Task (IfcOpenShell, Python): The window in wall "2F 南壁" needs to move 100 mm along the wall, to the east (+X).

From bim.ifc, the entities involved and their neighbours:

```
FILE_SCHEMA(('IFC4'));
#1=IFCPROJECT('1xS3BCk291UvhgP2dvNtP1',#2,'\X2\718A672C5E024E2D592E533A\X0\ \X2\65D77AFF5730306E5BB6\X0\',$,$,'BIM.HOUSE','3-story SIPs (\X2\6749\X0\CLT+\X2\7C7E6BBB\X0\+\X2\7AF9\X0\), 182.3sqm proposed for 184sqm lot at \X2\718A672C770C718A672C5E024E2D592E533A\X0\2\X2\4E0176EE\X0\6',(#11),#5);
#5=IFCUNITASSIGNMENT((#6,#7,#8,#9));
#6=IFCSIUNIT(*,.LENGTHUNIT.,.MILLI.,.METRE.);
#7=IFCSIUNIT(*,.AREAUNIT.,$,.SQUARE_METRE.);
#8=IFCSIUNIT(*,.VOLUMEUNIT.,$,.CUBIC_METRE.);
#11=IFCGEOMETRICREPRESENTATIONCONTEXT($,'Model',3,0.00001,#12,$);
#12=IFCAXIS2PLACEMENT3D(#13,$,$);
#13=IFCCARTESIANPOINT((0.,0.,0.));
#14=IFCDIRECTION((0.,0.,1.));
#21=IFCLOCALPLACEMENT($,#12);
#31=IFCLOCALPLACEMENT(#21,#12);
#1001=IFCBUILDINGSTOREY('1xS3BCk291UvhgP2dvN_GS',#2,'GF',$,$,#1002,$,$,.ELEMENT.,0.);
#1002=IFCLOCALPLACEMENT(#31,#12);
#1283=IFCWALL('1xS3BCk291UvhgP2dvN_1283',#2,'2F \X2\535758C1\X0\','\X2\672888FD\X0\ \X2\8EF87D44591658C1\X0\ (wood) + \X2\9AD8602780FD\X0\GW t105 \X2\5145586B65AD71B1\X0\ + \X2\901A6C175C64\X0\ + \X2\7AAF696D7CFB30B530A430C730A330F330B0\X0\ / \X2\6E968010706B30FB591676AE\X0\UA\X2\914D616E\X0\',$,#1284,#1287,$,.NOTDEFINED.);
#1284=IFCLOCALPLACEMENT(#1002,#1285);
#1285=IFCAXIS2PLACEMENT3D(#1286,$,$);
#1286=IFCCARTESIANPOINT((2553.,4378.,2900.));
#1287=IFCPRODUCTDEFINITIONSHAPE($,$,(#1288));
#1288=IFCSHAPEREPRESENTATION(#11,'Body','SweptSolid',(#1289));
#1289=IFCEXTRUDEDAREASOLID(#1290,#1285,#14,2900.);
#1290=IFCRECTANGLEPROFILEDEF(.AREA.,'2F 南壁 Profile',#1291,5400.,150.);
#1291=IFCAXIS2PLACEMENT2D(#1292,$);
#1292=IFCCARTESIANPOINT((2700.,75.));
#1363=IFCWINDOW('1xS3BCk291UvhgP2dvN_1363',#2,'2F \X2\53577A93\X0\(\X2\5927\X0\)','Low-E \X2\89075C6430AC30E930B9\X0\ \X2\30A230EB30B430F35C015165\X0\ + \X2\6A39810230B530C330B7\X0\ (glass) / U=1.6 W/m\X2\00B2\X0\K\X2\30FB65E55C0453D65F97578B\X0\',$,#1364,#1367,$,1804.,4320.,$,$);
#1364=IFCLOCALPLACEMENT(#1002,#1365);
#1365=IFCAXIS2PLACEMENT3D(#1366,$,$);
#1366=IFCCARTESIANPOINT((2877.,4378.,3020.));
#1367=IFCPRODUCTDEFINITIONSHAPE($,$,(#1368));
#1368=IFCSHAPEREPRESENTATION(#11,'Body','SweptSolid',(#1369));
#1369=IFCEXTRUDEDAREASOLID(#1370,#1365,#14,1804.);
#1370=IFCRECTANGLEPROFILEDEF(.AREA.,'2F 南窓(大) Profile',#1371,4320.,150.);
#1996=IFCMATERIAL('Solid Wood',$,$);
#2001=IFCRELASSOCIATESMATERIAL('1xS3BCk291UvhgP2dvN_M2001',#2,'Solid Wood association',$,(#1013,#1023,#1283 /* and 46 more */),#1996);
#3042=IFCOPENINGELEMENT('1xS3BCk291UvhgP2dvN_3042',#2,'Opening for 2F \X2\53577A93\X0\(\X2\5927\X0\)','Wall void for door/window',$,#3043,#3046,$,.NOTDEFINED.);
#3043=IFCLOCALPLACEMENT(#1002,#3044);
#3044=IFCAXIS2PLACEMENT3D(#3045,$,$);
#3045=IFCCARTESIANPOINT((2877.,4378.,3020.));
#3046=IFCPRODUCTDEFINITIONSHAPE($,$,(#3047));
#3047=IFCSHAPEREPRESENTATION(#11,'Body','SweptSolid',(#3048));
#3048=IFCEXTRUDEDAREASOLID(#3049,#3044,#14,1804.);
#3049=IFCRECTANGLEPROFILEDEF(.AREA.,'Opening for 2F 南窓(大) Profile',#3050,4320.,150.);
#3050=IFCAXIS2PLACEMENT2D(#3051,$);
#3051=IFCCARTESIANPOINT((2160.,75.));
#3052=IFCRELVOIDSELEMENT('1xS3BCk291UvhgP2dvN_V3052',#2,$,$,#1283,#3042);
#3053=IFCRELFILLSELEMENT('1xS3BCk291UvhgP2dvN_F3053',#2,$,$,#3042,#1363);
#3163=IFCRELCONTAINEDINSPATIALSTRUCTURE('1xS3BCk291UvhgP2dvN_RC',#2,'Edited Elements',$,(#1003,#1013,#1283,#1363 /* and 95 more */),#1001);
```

```python
import ifcopenshell
import ifcopenshell.api.geometry
import ifcopenshell.util.placement
import ifcopenshell.util.unit

model = ifcopenshell.open("bim.ifc")
unit_scale = ifcopenshell.util.unit.calculate_unit_scale(model)

window = model.by_guid("1xS3BCk291UvhgP2dvN_1363")
opening = window.FillsVoids[0].RelatingOpeningElement
wall = opening.VoidsElements[0].RelatingBuildingElement

wall_matrix = ifcopenshell.util.placement.get_local_placement(wall.ObjectPlacement)
shift = wall_matrix[:3, 0] * 0.1 / unit_scale
before = ifcopenshell.util.placement.get_local_placement(window.ObjectPlacement)[:3, 3].copy()

# The window is not placed relative to its opening, so move both.
for product in (opening, window):
    matrix = ifcopenshell.util.placement.get_local_placement(product.ObjectPlacement)
    matrix[:3, 3] += shift
    ifcopenshell.api.geometry.edit_object_placement(model, product=product, matrix=matrix, is_si=False)

after = ifcopenshell.util.placement.get_local_placement(window.ObjectPlacement)[:3, 3]
print("window moved by", (after - before).round(3) + 0.0)

model.write("bim-out.ifc")
```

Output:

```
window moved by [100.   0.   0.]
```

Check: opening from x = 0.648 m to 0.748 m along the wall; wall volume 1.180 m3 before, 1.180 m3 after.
